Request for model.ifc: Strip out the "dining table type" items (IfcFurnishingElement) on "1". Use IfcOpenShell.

First a look at what the model holds.

```python
import ifcopenshell
import ifcopenshell.util.element

model = ifcopenshell.open("model.ifc")
print(model.schema)
storey = next(s for s in model.by_type("IfcBuildingStorey") if s.Name == "1")
furniture = [e for e in ifcopenshell.util.element.get_decomposition(storey) if e.is_a("IfcFurnishingElement")]
seen = {}
for e in furniture:
    element_type = ifcopenshell.util.element.get_type(e)
    name = element_type.Name if element_type not in (None, e) else None
    seen[name] = seen.get(name, 0) + 1
for name, count in sorted(seen.items(), key=str):
    print(count, "x", name)
```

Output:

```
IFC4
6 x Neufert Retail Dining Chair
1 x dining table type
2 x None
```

```python
import ifcopenshell
import ifcopenshell.api.root
import ifcopenshell.util.element

model = ifcopenshell.open("model.ifc")

storey = next(s for s in model.by_type("IfcBuildingStorey") if s.Name == "1")
furniture = [e for e in ifcopenshell.util.element.get_decomposition(storey) if e.is_a("IfcFurnishingElement")]
targets = [e for e in furniture if (t := ifcopenshell.util.element.get_type(e)) not in (None, e) and t.Name == "dining table type"]

for e in targets:
    ifcopenshell.api.root.remove_product(model, product=e)
print(len(targets), "removed")

model.write("model_v2.ifc")
```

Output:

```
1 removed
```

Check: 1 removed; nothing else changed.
